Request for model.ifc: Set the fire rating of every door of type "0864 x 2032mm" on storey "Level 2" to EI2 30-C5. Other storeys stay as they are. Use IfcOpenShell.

First a look at what the model holds.

```python
import ifcopenshell
import ifcopenshell.util.element

model = ifcopenshell.open("model.ifc")
print(model.schema)
storey = next(s for s in model.by_type("IfcBuildingStorey") if s.Name == "Level 2")
doors = [e for e in ifcopenshell.util.element.get_decomposition(storey) if e.is_a("IfcDoor")]
seen = {}
for e in doors:
    element_type = ifcopenshell.util.element.get_type(e)
    key = (element_type.Name if element_type != e and element_type else None, ifcopenshell.util.element.get_pset(e, "Pset_DoorCommon", "FireRating"))
    seen[key] = seen.get(key, 0) + 1
for (name, value), count in sorted(seen.items(), key=str):
    print(count, "x", name, "|", value)
```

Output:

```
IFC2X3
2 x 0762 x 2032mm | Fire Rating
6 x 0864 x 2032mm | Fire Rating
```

```python
import ifcopenshell
import ifcopenshell.api.pset
import ifcopenshell.util.element

model = ifcopenshell.open("model.ifc")

storey = next(s for s in model.by_type("IfcBuildingStorey") if s.Name == "Level 2")
doors = [e for e in ifcopenshell.util.element.get_decomposition(storey) if e.is_a("IfcDoor")]

count = 0
for e in doors:
    element_type = ifcopenshell.util.element.get_type(e)
    if element_type in (None, e) or element_type.Name != "0864 x 2032mm":
        continue
    # add_pset returns the element's existing set when there is one.
    pset = ifcopenshell.api.pset.add_pset(model, product=e, name="Pset_DoorCommon")
    ifcopenshell.api.pset.edit_pset(model, pset=pset, properties={"FireRating": "EI2 30-C5"})
    count += 1

print(count, "doors updated")

model.write("model_rev.ifc")
```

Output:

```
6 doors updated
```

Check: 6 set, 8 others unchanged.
